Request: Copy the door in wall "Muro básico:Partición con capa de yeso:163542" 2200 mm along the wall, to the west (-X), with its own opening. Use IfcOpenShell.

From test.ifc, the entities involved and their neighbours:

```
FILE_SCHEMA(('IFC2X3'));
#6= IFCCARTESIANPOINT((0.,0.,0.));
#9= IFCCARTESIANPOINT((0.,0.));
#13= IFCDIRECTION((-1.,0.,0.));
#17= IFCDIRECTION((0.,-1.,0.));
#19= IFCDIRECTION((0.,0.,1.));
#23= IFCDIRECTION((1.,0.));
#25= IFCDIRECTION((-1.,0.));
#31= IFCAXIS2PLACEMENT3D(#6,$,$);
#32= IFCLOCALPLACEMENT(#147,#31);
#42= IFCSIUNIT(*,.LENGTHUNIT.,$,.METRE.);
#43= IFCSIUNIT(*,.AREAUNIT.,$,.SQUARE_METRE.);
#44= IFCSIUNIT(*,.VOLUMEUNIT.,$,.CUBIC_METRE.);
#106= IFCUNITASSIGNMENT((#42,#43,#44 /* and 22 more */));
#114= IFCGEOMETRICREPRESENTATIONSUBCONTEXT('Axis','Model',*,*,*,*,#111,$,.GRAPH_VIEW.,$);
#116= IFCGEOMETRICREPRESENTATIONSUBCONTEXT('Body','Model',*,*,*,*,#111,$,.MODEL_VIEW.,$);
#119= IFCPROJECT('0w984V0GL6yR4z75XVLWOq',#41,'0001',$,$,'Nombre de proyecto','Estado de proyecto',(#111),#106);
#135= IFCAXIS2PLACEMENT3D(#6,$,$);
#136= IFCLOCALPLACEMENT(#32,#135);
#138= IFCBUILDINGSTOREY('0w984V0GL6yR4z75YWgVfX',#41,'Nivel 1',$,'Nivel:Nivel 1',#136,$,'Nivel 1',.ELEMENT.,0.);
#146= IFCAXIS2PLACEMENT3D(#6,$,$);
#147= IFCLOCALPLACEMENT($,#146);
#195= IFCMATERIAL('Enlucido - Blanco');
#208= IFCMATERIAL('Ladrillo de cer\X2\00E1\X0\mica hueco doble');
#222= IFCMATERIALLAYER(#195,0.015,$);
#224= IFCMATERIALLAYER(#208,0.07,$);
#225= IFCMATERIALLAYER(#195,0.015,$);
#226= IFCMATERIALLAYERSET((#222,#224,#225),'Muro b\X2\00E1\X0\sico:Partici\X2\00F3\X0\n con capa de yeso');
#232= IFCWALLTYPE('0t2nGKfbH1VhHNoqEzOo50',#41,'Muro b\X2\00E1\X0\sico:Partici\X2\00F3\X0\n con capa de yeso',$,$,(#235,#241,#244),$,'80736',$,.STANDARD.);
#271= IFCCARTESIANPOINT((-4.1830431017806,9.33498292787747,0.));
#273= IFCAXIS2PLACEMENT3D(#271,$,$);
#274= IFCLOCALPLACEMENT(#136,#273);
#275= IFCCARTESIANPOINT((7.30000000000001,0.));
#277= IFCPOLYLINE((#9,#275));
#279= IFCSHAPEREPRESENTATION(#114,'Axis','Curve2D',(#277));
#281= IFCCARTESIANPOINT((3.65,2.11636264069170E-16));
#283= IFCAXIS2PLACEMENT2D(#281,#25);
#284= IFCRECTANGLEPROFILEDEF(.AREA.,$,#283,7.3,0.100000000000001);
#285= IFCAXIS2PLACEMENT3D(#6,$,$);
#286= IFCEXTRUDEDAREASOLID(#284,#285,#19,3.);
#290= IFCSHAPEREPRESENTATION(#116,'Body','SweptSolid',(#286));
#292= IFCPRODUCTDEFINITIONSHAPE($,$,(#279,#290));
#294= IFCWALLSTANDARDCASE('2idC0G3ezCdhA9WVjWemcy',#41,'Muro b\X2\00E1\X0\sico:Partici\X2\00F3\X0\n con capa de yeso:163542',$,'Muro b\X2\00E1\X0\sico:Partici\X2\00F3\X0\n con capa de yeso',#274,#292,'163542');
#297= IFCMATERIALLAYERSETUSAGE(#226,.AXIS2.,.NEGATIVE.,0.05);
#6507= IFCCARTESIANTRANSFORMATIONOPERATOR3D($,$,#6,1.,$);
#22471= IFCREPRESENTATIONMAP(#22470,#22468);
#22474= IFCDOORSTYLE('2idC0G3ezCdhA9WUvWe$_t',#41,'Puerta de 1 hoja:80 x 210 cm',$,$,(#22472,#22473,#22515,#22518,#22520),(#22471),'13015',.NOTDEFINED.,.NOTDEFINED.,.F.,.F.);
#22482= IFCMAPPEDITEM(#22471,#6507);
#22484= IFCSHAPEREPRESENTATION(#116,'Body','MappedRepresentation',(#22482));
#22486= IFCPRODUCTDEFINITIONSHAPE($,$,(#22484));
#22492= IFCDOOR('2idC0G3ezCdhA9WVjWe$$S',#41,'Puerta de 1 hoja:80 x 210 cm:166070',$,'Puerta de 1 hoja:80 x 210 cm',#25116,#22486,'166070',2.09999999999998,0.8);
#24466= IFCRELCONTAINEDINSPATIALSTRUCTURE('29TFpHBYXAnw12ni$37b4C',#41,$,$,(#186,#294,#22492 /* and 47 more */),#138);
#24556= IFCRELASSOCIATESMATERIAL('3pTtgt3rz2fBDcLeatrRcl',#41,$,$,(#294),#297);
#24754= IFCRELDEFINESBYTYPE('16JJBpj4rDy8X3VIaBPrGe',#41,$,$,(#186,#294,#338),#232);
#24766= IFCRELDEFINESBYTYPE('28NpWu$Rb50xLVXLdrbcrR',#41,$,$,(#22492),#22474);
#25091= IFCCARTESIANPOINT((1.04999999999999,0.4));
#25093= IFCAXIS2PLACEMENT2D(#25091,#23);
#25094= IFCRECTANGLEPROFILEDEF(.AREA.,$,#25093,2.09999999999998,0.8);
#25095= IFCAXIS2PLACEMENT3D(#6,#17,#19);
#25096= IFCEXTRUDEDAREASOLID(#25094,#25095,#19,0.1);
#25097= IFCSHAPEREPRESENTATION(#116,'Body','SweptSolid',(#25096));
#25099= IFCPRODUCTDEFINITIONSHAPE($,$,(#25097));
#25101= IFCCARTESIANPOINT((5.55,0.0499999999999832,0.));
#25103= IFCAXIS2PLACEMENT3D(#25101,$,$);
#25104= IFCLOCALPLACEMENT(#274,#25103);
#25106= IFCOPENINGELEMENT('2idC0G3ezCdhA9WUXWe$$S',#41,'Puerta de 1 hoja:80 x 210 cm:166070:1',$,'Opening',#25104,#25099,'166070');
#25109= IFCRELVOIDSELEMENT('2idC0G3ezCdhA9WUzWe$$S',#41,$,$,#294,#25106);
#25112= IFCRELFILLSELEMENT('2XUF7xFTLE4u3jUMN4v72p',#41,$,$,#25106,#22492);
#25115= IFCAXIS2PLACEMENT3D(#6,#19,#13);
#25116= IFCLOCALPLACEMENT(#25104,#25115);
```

```python
import ifcopenshell
import ifcopenshell.api.feature
import ifcopenshell.api.geometry
import ifcopenshell.api.root
import ifcopenshell.geom
import ifcopenshell.util.element
import ifcopenshell.util.placement
import ifcopenshell.util.shape

model = ifcopenshell.open("test.ifc")
settings = ifcopenshell.geom.settings()


def volume(element):
    """Net volume in cubic metres, openings subtracted."""
    shape = ifcopenshell.geom.create_shape(settings, element)
    return ifcopenshell.util.shape.get_volume(shape.geometry)


def reuse_history(source, copy):
    """copy_class also copies each property set's owner history, people and application; keep the originals."""
    for rel in copy.IsDefinedBy:
        if rel.is_a("IfcRelDefinesByProperties") and (history := rel.RelatingPropertyDefinition.OwnerHistory):
            rel.RelatingPropertyDefinition.OwnerHistory = source.OwnerHistory
            ifcopenshell.util.element.remove_deep2(model, history)


door = model.by_id(22492)
opening = door.FillsVoids[0].RelatingOpeningElement
wall = opening.VoidsElements[0].RelatingBuildingElement
before = volume(wall)
shift = ifcopenshell.util.placement.get_local_placement(wall.ObjectPlacement)[:3, 0] * -2.2

# copy_class copies the void relationship, type, container and properties, but no geometry.
new_opening = ifcopenshell.api.root.copy_class(model, product=opening)
new_opening.Representation = ifcopenshell.util.element.copy_deep(
    model, opening.Representation, exclude=["IfcGeometricRepresentationContext", "IfcRepresentationMap"]
)
new_opening.Name = "Puerta de 1 hoja:80 x 210 cm"
new_opening.Tag = None
new_door = ifcopenshell.api.root.copy_class(model, product=door)
new_door.Representation = ifcopenshell.util.element.copy_deep(
    model, door.Representation, exclude=["IfcGeometricRepresentationContext", "IfcRepresentationMap"]
)
new_door.Name = "Puerta de 1 hoja:80 x 210 cm"
new_door.Tag = None
reuse_history(door, new_door)
fills = ifcopenshell.api.feature.add_filling(model, opening=new_opening, element=new_door)
fills.OwnerHistory = new_door.OwnerHistory  # required in IFC2X3

for old, new in ((opening, new_opening), (door, new_door)):
    matrix = ifcopenshell.util.placement.get_local_placement(old.ObjectPlacement)
    matrix[:3, 3] += shift
    ifcopenshell.api.geometry.edit_object_placement(model, product=new, matrix=matrix, is_si=False)

after = volume(wall)

print(f"wall volume {before:.3f} -> {after:.3f} m3")

model.write("test_edited.ifc")
```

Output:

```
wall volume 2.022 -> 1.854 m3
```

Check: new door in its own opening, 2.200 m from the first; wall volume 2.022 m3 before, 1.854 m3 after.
